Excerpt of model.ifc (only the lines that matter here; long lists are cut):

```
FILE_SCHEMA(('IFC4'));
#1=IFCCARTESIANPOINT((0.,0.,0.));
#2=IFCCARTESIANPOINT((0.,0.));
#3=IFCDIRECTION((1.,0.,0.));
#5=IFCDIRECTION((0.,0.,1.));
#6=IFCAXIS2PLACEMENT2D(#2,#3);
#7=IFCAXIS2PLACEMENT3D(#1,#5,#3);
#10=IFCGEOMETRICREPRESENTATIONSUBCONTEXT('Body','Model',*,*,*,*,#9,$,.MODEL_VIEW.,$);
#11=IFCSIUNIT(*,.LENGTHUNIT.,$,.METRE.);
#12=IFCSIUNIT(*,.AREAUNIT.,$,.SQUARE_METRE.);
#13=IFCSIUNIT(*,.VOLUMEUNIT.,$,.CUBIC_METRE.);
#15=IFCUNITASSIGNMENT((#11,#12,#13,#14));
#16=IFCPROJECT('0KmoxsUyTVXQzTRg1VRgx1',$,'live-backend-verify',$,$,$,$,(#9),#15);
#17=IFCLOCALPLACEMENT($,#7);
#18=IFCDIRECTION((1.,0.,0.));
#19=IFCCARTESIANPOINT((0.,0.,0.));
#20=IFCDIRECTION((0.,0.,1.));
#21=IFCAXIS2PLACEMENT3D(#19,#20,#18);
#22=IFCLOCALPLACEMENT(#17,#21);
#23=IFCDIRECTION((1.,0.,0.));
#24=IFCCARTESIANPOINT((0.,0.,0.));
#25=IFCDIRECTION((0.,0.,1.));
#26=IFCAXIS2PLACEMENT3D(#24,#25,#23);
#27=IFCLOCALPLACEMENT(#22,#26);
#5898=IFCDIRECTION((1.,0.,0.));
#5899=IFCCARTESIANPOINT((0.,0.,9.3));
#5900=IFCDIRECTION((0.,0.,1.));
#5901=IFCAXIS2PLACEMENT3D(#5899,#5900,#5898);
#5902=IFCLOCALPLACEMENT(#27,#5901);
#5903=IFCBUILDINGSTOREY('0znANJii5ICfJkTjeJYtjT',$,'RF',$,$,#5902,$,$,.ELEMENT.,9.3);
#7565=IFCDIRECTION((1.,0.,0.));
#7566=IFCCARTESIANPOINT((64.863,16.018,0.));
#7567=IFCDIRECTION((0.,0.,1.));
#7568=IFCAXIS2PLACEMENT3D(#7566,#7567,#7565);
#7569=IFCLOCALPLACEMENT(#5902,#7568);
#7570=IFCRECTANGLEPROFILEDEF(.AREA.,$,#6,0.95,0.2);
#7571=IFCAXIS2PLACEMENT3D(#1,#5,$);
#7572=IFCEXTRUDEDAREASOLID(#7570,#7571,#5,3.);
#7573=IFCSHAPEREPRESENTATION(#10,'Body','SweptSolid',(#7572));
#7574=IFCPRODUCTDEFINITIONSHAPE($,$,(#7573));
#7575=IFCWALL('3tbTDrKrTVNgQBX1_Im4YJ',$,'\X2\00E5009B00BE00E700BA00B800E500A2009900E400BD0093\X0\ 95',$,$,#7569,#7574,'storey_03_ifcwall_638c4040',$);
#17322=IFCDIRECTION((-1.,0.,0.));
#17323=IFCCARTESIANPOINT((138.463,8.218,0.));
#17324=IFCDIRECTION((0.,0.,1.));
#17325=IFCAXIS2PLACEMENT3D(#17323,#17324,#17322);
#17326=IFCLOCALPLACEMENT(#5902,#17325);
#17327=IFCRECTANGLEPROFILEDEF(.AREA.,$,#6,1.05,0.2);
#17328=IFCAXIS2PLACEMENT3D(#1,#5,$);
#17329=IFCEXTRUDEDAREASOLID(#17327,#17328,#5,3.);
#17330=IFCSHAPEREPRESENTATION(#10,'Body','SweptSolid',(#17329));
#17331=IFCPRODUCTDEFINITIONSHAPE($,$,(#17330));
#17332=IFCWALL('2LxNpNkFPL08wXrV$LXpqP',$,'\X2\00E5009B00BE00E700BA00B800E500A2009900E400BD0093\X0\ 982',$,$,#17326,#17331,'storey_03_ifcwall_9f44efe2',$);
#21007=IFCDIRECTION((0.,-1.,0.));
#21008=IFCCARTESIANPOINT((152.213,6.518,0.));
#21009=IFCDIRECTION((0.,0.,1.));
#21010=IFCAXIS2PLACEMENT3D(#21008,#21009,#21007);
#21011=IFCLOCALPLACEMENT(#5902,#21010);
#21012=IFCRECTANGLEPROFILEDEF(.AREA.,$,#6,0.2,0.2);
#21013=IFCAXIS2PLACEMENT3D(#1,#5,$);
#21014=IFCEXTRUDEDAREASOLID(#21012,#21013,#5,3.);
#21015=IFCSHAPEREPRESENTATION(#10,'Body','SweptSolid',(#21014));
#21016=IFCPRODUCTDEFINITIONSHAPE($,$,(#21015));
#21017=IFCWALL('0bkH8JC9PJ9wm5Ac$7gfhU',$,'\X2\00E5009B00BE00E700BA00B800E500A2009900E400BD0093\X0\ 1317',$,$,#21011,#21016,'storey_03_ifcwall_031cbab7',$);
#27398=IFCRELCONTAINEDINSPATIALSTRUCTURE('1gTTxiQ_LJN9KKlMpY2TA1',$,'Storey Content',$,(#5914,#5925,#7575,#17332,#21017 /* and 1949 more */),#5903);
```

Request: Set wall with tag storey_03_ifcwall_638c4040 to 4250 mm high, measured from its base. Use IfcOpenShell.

```python
import ifcopenshell
import ifcopenshell.geom
import ifcopenshell.util.representation
import ifcopenshell.util.shape
import ifcopenshell.util.unit

model = ifcopenshell.open("model.ifc")
unit_scale = ifcopenshell.util.unit.calculate_unit_scale(model)
settings = ifcopenshell.geom.settings()


def volume(element):
    """Net volume in cubic metres, openings subtracted."""
    shape = ifcopenshell.geom.create_shape(settings, element)
    return ifcopenshell.util.shape.get_volume(shape.geometry)


wall = model.by_guid("3tbTDrKrTVNgQBX1_Im4YJ")
before = volume(wall)

body = ifcopenshell.util.representation.get_representation(wall, "Model", "Body")
solid = body.Items[0]
old_height = solid.Depth
solid.Depth = 4.25 / unit_scale
after = volume(wall)

print(f"height {old_height:g} -> {solid.Depth:g}, volume {before:.3f} -> {after:.3f} m3")

model.write("model_updated.ifc")
```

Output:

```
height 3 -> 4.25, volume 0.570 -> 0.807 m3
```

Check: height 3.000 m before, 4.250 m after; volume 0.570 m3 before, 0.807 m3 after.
